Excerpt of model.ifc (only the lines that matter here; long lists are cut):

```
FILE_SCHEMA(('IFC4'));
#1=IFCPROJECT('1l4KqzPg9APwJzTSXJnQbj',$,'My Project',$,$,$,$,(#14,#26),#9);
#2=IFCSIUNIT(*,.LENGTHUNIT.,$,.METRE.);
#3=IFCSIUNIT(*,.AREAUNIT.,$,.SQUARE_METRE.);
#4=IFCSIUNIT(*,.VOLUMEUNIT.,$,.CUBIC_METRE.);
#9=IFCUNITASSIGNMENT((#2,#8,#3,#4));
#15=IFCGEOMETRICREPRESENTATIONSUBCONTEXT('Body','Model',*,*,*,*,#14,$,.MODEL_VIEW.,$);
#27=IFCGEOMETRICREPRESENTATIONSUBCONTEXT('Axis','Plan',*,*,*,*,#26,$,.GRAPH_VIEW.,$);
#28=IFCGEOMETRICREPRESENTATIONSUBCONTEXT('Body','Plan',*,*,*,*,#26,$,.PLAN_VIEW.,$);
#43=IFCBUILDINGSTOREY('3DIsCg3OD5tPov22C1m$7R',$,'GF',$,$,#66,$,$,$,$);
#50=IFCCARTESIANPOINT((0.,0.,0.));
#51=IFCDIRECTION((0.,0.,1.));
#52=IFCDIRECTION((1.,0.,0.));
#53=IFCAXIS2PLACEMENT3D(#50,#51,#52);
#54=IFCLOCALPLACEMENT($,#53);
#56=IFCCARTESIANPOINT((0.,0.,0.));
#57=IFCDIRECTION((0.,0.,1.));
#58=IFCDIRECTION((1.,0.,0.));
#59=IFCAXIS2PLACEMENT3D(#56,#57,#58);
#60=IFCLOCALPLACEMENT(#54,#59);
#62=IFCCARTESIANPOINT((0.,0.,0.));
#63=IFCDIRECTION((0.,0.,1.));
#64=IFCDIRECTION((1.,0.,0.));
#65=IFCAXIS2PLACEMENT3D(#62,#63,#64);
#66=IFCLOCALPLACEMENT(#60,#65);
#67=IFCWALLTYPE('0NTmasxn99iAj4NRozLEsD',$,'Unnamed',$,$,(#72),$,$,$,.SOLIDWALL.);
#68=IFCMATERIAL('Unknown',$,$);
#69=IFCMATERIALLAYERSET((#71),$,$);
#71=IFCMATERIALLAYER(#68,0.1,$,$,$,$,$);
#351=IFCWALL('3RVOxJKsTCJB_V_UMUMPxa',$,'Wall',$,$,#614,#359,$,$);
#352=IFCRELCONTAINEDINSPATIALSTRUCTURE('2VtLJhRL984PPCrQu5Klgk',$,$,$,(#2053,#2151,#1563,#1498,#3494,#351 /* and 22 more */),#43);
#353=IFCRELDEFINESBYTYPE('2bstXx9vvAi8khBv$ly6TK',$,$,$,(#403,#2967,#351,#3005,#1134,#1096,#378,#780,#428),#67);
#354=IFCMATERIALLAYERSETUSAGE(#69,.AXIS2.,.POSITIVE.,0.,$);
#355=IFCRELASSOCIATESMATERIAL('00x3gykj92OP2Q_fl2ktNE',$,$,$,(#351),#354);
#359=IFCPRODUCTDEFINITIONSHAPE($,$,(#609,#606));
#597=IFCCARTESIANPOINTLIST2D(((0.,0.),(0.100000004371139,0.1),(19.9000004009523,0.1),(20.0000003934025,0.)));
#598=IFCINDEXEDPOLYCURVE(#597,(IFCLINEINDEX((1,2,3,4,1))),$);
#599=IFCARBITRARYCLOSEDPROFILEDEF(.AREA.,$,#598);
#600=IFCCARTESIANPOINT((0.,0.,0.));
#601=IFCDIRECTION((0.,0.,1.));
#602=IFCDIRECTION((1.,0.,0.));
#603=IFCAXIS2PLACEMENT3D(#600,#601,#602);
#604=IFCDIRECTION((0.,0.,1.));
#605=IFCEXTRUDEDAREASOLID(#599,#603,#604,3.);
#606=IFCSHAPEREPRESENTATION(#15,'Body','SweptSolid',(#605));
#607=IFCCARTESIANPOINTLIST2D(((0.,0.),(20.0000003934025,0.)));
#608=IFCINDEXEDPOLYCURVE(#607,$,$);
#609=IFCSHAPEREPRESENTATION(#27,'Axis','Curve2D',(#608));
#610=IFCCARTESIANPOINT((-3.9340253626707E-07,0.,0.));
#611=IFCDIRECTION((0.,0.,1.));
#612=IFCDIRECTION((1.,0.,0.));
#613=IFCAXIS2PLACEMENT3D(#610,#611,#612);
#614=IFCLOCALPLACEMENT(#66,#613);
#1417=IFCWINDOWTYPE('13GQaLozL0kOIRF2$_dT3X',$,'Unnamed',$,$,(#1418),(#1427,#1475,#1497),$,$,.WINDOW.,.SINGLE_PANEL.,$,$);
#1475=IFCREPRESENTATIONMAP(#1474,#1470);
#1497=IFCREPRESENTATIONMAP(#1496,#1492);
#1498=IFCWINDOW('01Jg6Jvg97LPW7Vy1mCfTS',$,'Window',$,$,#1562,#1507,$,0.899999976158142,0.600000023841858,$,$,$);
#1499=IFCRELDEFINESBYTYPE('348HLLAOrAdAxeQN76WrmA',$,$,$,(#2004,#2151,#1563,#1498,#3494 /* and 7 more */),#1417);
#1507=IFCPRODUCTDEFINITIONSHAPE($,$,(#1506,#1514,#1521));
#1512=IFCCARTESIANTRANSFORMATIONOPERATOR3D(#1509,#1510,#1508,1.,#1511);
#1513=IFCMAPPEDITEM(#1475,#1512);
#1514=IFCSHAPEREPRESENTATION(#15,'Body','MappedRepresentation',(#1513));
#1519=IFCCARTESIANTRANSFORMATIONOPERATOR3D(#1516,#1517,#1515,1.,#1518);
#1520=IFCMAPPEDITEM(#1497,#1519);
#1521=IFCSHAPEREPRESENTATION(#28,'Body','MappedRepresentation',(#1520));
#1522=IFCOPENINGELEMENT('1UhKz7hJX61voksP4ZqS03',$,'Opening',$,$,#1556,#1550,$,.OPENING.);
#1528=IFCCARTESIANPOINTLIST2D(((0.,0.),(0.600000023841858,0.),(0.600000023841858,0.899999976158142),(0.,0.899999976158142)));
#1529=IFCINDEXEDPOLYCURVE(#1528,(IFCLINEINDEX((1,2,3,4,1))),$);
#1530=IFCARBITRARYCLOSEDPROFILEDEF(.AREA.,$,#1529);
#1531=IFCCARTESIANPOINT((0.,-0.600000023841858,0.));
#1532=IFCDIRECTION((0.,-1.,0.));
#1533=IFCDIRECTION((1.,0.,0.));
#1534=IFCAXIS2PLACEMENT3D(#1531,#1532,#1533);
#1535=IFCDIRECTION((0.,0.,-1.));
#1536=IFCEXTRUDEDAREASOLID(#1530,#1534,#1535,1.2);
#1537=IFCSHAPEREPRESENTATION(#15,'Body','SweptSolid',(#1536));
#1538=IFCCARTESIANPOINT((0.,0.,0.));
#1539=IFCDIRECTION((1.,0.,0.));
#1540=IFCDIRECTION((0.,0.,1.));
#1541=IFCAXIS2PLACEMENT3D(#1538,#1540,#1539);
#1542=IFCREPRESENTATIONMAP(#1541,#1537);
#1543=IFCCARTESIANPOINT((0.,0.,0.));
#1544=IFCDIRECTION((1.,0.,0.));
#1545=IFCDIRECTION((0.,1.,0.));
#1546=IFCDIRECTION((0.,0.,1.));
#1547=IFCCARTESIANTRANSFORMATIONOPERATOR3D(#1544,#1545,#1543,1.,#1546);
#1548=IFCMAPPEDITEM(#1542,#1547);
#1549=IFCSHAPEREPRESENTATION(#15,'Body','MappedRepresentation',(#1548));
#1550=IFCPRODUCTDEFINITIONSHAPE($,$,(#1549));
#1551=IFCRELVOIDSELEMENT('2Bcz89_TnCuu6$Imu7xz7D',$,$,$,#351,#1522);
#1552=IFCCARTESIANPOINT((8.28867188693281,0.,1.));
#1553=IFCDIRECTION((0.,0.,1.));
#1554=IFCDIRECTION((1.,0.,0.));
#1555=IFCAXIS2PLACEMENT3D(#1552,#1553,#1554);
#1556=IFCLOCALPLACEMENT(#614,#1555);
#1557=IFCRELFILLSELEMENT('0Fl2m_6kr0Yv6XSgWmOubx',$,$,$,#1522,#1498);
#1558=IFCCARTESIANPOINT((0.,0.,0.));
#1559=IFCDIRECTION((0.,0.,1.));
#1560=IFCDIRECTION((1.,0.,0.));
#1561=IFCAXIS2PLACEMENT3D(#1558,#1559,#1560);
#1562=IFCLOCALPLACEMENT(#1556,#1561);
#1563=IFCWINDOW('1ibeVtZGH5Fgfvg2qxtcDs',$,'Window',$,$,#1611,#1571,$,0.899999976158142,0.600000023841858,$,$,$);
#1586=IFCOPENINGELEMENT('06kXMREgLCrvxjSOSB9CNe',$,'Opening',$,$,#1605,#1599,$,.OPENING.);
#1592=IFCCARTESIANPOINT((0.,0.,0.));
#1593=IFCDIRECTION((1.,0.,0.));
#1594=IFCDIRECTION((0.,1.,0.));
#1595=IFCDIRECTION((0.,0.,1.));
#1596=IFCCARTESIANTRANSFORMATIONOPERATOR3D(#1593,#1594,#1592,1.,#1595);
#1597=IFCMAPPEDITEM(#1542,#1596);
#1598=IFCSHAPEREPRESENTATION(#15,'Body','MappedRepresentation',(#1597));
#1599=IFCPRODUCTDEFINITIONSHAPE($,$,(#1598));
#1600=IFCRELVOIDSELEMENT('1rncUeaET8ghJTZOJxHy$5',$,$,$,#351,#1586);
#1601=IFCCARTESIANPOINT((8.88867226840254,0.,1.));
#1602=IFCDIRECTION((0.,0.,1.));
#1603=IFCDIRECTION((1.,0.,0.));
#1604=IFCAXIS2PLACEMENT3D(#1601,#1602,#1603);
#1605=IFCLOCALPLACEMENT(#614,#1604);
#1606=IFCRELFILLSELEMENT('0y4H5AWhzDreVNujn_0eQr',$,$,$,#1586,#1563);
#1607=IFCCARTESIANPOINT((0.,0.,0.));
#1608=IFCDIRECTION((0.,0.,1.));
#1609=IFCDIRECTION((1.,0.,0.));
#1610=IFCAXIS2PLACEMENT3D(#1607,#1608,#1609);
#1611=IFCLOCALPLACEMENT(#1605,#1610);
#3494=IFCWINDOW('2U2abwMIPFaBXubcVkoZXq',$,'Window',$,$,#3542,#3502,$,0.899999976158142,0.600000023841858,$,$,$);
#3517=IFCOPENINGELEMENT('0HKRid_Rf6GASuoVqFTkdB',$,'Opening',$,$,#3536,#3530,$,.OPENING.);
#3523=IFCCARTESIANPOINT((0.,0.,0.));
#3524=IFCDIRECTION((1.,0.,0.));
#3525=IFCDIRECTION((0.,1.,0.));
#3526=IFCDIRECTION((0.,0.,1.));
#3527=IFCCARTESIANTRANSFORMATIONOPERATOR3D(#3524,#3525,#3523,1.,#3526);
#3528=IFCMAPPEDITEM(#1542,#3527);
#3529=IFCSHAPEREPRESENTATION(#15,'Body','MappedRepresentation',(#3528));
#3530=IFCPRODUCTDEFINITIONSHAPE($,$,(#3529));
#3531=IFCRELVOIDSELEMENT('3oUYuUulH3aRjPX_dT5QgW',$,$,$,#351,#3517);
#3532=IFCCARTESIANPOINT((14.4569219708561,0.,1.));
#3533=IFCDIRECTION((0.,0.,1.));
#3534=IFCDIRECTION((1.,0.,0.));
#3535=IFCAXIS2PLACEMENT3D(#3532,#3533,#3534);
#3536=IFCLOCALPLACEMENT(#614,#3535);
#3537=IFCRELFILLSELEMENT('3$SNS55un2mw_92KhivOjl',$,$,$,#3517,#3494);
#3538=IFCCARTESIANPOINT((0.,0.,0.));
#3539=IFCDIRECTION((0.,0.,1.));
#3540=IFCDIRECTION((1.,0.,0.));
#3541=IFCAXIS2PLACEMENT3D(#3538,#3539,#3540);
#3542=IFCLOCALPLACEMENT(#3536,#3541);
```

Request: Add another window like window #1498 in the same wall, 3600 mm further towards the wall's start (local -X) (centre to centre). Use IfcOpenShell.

```python
import ifcopenshell
import ifcopenshell.api.feature
import ifcopenshell.api.geometry
import ifcopenshell.api.root
import ifcopenshell.geom
import ifcopenshell.util.element
import ifcopenshell.util.placement
import ifcopenshell.util.shape

model = ifcopenshell.open("model.ifc")
settings = ifcopenshell.geom.settings()


def volume(element):
    """Net volume in cubic metres, openings subtracted."""
    shape = ifcopenshell.geom.create_shape(settings, element)
    return ifcopenshell.util.shape.get_volume(shape.geometry)


window = model.by_guid("01Jg6Jvg97LPW7Vy1mCfTS")
opening = window.FillsVoids[0].RelatingOpeningElement
wall = opening.VoidsElements[0].RelatingBuildingElement
before = volume(wall)
shift = ifcopenshell.util.placement.get_local_placement(wall.ObjectPlacement)[:3, 0] * -3.6

# copy_class copies the void relationship, type, container and properties, but no geometry.
new_opening = ifcopenshell.api.root.copy_class(model, product=opening)
new_opening.Representation = ifcopenshell.util.element.copy_deep(
    model, opening.Representation, exclude=["IfcGeometricRepresentationContext", "IfcRepresentationMap"]
)
new_window = ifcopenshell.api.root.copy_class(model, product=window)
new_window.Representation = ifcopenshell.util.element.copy_deep(
    model, window.Representation, exclude=["IfcGeometricRepresentationContext", "IfcRepresentationMap"]
)
ifcopenshell.api.feature.add_filling(model, opening=new_opening, element=new_window)

for old, new in ((opening, new_opening), (window, new_window)):
    matrix = ifcopenshell.util.placement.get_local_placement(old.ObjectPlacement)
    matrix[:3, 3] += shift
    ifcopenshell.api.geometry.edit_object_placement(model, product=new, matrix=matrix, is_si=False)

after = volume(wall)

print(f"wall volume {before:.3f} -> {after:.3f} m3")

model.write("model-out.ifc")
```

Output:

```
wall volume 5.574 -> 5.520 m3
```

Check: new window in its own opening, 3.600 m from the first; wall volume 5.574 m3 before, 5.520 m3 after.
